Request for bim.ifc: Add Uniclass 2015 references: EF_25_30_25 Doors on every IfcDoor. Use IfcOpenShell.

First a look at what the model holds.

```python
import ifcopenshell

model = ifcopenshell.open("bim.ifc")
print(model.schema)
print("classifications:", [c.Name for c in model.by_type("IfcClassification")])
for ifc_class in ("IfcDoor", "IfcRoof", "IfcStair", "IfcWall", "IfcWindow"):
    print(ifc_class, len(model.by_type(ifc_class)))
```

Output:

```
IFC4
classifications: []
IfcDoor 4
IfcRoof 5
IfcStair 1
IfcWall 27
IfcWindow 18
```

```python
import ifcopenshell
import ifcopenshell.api.classification

model = ifcopenshell.open("bim.ifc")

system = ifcopenshell.api.classification.add_classification(model, classification="Uniclass 2015")

codes = {
    "IfcDoor": ("EF_25_30_25", "Doors"),
}
for ifc_class, (code, name) in codes.items():
    products = model.by_type(ifc_class)
    ifcopenshell.api.classification.add_reference(
        model, products=products, classification=system, identification=code, name=name
    )
    print(code, len(products))

model.write("bim_v2.ifc")
```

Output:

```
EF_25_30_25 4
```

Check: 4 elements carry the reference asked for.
